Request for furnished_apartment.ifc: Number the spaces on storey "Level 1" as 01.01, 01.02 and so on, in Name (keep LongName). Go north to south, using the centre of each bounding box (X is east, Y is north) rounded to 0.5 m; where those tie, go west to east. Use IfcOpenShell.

First a look at what the model holds.

```python
import ifcopenshell
import ifcopenshell.util.element
import ifcopenshell.util.placement

model = ifcopenshell.open("furnished_apartment.ifc")
print(model.schema)
storey = next(s for s in model.by_type("IfcBuildingStorey") if s.Name == "Level 1")
spaces = [e for e in ifcopenshell.util.element.get_decomposition(storey) if e.is_a("IfcSpace")]
for e in sorted(spaces, key=lambda e: e.id()):
    origin = ifcopenshell.util.placement.get_local_placement(e.ObjectPlacement)[:3, 3]
    print(e.id(), e.Name, e.LongName, origin.round(2) + 0.0, sep=" | ")
```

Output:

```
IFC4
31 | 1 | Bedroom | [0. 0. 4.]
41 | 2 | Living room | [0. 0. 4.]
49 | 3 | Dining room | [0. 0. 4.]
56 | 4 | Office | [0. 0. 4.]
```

```python
import ifcopenshell
import ifcopenshell.geom
import ifcopenshell.util.element
import ifcopenshell.util.shape

model = ifcopenshell.open("furnished_apartment.ifc")
settings = ifcopenshell.geom.settings()
settings.set("use-world-coords", True)


def centre(element):
    shape = ifcopenshell.geom.create_shape(settings, element)
    return ifcopenshell.util.shape.get_bbox_centroid(shape.geometry)


storey = next(s for s in model.by_type("IfcBuildingStorey") if s.Name == "Level 1")
spaces = [e for e in ifcopenshell.util.element.get_decomposition(storey) if e.is_a("IfcSpace")]

# Insertion points can sit at a corner or the storey origin, so sort by the geometry (in metres).
centres = {e: centre(e) for e in spaces}
spaces.sort(key=lambda e: (-round(centres[e][1] / 0.5), centres[e][0]))

for i, e in enumerate(spaces, start=1):
    number = f"01.{i:02d}"
    e.Name = number
    print(e.id(), number)

model.write("furnished_apartment_edited.ifc")
```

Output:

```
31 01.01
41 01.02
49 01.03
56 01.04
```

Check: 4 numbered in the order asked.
